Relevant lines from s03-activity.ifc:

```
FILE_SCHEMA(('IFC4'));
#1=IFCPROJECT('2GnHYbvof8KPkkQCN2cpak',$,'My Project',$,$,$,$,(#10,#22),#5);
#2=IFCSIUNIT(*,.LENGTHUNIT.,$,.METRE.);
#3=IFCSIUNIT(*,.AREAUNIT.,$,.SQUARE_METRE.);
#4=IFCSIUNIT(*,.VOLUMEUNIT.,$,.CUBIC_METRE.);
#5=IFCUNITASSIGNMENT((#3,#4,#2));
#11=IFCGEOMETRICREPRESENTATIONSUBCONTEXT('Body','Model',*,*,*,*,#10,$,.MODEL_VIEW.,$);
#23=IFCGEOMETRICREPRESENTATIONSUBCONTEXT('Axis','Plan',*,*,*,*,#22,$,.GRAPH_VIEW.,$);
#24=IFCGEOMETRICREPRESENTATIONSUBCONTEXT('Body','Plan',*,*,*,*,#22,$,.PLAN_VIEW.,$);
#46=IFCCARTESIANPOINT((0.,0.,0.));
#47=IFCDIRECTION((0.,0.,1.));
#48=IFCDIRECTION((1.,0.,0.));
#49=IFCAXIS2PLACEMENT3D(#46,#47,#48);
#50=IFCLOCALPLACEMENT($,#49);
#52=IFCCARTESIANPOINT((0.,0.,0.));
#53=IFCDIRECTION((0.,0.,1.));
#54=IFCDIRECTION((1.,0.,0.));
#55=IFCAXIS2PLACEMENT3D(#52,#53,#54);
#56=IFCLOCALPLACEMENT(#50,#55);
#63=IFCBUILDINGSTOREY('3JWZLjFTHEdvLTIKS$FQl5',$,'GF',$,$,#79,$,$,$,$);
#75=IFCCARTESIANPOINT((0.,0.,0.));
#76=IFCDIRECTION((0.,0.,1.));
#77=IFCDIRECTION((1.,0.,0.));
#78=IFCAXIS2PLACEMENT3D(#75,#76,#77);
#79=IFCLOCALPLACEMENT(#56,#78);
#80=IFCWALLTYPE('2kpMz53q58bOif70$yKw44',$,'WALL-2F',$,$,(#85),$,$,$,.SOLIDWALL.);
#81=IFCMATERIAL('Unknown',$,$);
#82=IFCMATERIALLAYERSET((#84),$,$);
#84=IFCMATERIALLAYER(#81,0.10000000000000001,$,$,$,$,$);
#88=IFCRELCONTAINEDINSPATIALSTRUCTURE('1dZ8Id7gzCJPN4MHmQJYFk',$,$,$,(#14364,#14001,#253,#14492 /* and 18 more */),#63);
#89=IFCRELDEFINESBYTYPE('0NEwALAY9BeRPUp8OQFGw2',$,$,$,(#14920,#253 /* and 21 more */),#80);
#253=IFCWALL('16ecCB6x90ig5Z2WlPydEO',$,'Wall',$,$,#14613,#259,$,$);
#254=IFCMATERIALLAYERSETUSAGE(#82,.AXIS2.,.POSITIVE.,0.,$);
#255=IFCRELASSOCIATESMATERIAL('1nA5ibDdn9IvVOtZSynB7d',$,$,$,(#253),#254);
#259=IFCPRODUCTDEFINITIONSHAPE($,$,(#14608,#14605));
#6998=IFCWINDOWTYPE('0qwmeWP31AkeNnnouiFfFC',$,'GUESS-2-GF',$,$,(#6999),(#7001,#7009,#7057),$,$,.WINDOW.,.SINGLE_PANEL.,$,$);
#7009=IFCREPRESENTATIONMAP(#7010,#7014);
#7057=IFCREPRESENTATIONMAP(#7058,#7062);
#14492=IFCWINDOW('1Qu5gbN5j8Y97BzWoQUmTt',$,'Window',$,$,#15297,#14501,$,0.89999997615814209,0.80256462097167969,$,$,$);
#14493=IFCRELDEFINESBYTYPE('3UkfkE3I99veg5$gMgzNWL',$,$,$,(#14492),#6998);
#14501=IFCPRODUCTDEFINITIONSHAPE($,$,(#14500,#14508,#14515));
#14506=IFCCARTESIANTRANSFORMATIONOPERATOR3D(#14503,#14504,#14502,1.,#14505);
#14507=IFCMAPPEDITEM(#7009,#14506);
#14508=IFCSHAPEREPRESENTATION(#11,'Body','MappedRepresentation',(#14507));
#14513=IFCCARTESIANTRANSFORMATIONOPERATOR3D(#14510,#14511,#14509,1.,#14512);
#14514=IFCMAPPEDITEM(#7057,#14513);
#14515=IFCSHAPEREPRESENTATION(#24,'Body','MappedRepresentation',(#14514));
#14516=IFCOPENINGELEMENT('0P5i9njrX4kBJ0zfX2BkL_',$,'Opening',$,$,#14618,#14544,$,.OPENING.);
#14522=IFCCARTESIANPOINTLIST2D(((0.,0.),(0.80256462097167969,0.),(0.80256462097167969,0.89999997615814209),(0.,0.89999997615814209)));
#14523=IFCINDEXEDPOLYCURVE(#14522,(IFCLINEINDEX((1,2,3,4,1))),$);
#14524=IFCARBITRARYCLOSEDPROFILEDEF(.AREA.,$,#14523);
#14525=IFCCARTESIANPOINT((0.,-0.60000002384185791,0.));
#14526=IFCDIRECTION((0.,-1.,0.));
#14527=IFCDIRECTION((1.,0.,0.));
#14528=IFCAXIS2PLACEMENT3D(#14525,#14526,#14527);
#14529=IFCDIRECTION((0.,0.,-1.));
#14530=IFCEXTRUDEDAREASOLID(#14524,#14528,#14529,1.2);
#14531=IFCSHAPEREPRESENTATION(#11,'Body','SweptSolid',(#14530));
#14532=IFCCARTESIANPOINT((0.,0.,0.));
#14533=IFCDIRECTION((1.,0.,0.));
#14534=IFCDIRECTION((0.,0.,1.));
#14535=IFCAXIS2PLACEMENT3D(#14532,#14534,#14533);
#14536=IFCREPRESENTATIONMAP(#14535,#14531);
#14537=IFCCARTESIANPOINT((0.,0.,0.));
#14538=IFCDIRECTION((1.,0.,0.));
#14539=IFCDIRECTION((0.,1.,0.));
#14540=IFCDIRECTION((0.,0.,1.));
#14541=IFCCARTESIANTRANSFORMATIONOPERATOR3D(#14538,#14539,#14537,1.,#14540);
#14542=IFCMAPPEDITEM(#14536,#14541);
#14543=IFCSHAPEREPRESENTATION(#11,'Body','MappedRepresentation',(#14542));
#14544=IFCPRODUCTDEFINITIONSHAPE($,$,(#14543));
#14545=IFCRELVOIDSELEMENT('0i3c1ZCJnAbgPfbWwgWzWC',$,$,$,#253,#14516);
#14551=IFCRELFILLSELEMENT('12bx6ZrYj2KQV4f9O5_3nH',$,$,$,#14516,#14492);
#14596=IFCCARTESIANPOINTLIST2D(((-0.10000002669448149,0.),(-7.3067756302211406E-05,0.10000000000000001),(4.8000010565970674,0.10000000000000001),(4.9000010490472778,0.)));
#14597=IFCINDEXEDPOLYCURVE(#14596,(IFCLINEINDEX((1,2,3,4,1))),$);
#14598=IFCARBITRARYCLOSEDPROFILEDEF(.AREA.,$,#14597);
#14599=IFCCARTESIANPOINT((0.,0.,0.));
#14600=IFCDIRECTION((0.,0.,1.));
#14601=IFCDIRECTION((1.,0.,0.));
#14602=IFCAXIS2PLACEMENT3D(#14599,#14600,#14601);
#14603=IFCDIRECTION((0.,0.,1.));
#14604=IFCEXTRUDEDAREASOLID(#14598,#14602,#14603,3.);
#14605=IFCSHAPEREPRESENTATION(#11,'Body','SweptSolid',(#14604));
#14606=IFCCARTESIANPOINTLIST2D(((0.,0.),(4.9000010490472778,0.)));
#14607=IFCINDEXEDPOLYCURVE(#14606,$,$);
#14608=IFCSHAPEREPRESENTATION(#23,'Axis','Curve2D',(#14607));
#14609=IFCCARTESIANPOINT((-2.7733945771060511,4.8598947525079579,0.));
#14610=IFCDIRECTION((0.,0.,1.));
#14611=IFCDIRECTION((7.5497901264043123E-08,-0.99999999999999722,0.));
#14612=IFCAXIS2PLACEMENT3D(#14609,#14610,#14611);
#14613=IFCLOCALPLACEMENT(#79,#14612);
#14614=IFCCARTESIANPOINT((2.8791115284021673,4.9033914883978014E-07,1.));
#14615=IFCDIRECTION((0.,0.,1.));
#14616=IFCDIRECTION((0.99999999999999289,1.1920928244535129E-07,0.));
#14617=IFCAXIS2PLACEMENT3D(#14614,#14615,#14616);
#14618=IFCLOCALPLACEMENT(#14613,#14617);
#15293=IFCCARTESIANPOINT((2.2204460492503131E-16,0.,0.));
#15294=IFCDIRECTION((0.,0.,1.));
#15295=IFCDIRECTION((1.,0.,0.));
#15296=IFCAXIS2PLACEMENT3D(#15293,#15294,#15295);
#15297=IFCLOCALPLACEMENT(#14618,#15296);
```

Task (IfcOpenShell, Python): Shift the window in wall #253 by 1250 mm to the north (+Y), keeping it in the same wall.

```python
import ifcopenshell
import ifcopenshell.api.geometry
import ifcopenshell.util.placement

model = ifcopenshell.open("s03-activity.ifc")

window = model.by_id(14492)
opening = window.FillsVoids[0].RelatingOpeningElement
wall = opening.VoidsElements[0].RelatingBuildingElement

wall_matrix = ifcopenshell.util.placement.get_local_placement(wall.ObjectPlacement)
shift = wall_matrix[:3, 0] * -1.25
before = ifcopenshell.util.placement.get_local_placement(window.ObjectPlacement)[:3, 3].copy()

# The window is placed relative to its opening, so it follows when the opening moves.
matrix = ifcopenshell.util.placement.get_local_placement(opening.ObjectPlacement)
matrix[:3, 3] += shift
ifcopenshell.api.geometry.edit_object_placement(
    model, product=opening, matrix=matrix, is_si=False, should_transform_children=True
)

after = ifcopenshell.util.placement.get_local_placement(window.ObjectPlacement)[:3, 3]
print("window moved by", (after - before).round(3) + 0.0)

model.write("s03-activity-out.ifc")
```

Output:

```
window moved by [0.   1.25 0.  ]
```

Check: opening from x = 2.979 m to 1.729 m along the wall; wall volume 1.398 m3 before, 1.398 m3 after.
